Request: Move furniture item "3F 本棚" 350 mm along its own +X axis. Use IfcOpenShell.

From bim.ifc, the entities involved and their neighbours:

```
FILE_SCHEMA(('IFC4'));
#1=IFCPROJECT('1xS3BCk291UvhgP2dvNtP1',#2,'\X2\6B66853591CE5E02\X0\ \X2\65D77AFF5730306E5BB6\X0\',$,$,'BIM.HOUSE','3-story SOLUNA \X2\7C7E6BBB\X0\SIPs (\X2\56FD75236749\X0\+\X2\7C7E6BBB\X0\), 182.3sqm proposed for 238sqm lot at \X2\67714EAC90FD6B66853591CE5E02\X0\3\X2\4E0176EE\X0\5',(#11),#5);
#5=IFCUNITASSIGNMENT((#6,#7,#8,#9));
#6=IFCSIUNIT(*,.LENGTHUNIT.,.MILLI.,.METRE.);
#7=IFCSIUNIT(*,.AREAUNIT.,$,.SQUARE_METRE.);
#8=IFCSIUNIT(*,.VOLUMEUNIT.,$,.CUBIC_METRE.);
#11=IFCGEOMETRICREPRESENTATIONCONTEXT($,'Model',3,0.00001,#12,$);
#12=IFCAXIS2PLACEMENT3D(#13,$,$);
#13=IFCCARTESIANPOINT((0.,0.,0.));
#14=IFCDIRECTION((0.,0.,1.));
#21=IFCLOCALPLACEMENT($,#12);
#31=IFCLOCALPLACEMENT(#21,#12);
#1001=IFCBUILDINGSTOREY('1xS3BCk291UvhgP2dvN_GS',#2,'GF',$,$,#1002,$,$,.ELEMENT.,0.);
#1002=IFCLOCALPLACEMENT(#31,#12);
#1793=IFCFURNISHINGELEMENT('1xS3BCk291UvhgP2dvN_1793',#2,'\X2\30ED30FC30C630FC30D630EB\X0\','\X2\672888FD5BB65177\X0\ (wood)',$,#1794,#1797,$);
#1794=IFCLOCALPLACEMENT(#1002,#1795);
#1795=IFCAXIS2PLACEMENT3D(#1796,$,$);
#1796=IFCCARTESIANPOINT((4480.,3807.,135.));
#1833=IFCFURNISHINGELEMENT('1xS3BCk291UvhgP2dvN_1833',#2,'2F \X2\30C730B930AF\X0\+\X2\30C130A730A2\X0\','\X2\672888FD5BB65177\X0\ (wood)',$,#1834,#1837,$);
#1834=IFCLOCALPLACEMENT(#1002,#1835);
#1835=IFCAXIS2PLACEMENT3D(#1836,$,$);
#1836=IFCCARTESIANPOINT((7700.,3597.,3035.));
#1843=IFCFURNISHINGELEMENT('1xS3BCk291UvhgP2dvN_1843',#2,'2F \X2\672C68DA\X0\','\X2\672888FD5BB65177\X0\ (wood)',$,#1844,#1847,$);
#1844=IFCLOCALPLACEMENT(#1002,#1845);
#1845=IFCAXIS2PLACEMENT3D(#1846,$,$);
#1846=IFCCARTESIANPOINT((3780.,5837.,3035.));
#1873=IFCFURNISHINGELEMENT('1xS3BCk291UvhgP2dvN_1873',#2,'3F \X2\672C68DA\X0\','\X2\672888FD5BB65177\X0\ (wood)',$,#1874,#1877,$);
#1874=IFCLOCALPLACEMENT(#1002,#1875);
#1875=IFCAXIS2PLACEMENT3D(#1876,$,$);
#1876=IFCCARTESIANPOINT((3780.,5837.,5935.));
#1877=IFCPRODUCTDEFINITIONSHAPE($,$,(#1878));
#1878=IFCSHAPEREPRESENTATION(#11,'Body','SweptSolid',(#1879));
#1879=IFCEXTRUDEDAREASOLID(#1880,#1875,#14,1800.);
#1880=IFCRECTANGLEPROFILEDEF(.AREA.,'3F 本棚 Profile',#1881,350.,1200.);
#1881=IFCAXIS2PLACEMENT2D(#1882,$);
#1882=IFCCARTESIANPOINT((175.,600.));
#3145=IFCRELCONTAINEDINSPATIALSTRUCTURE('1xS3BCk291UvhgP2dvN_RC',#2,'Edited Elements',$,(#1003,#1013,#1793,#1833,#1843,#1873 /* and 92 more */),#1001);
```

```python
import ifcopenshell
import ifcopenshell.api.geometry
import ifcopenshell.util.placement
import ifcopenshell.util.unit

model = ifcopenshell.open("bim.ifc")
unit_scale = ifcopenshell.util.unit.calculate_unit_scale(model)

item = model.by_id(1873)
matrix = ifcopenshell.util.placement.get_local_placement(item.ObjectPlacement)
matrix[:3, 3] += matrix[:3, 0] * 0.35 / unit_scale
ifcopenshell.api.geometry.edit_object_placement(model, product=item, matrix=matrix, is_si=False)

print(ifcopenshell.util.placement.get_local_placement(item.ObjectPlacement).round(3) + 0.0)

model.write("bim_updated.ifc")
```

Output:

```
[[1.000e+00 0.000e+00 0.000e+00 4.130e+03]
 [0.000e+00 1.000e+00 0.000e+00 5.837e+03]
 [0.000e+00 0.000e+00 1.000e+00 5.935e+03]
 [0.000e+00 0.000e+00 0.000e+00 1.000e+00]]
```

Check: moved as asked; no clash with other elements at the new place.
